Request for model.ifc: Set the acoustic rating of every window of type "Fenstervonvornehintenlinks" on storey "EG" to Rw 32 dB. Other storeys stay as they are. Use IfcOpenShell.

First a look at what the model holds.

```python
import ifcopenshell
import ifcopenshell.util.element

model = ifcopenshell.open("model.ifc")
print(model.schema)
storey = next(s for s in model.by_type("IfcBuildingStorey") if s.Name == "EG")
windows = [e for e in ifcopenshell.util.element.get_decomposition(storey) if e.is_a("IfcWindow")]
seen = {}
for e in windows:
    element_type = ifcopenshell.util.element.get_type(e)
    key = (element_type.Name if element_type != e and element_type else None, ifcopenshell.util.element.get_pset(e, "Pset_WindowCommon", "AcousticRating"))
    seen[key] = seen.get(key, 0) + 1
for (name, value), count in sorted(seen.items(), key=str):
    print(count, "x", name, "|", value)
```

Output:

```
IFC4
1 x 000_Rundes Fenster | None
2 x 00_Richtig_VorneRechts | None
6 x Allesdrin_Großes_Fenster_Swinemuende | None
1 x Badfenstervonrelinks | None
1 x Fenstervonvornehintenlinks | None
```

```python
import ifcopenshell
import ifcopenshell.api.pset
import ifcopenshell.util.element

model = ifcopenshell.open("model.ifc")

storey = next(s for s in model.by_type("IfcBuildingStorey") if s.Name == "EG")
windows = [e for e in ifcopenshell.util.element.get_decomposition(storey) if e.is_a("IfcWindow")]

count = 0
for e in windows:
    element_type = ifcopenshell.util.element.get_type(e)
    if element_type in (None, e) or element_type.Name != "Fenstervonvornehintenlinks":
        continue
    # add_pset returns the element's existing set when there is one.
    pset = ifcopenshell.api.pset.add_pset(model, product=e, name="Pset_WindowCommon")
    ifcopenshell.api.pset.edit_pset(model, pset=pset, properties={"AcousticRating": "Rw 32 dB"})
    count += 1

print(count, "windows updated")

model.write("model_v2.ifc")
```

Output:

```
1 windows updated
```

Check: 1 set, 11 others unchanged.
